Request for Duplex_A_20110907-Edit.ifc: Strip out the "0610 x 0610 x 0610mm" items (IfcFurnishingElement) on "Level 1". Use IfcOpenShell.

First a look at what the model holds.

```python
import ifcopenshell
import ifcopenshell.util.element

model = ifcopenshell.open("Duplex_A_20110907-Edit.ifc")
print(model.schema)
storey = next(s for s in model.by_type("IfcBuildingStorey") if s.Name == "Level 1")
furniture = [e for e in ifcopenshell.util.element.get_decomposition(storey) if e.is_a("IfcFurnishingElement")]
seen = {}
for e in furniture:
    element_type = ifcopenshell.util.element.get_type(e)
    name = element_type.Name if element_type not in (None, e) else None
    seen[name] = seen.get(name, 0) + 1
for name, count in sorted(seen.items(), key=str):
    print(count, "x", name)
```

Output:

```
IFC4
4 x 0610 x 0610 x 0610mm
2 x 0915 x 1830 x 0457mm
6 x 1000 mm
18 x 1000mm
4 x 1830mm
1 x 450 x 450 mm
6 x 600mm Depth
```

```python
import ifcopenshell
import ifcopenshell.api.root
import ifcopenshell.util.element

model = ifcopenshell.open("Duplex_A_20110907-Edit.ifc")

storey = next(s for s in model.by_type("IfcBuildingStorey") if s.Name == "Level 1")
furniture = [e for e in ifcopenshell.util.element.get_decomposition(storey) if e.is_a("IfcFurnishingElement")]
targets = [e for e in furniture if (t := ifcopenshell.util.element.get_type(e)) not in (None, e) and t.Name == "0610 x 0610 x 0610mm"]

for e in targets:
    ifcopenshell.api.root.remove_product(model, product=e)
print(len(targets), "removed")

model.write("Duplex_A_20110907-Edit-out.ifc")
```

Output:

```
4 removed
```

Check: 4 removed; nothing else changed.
